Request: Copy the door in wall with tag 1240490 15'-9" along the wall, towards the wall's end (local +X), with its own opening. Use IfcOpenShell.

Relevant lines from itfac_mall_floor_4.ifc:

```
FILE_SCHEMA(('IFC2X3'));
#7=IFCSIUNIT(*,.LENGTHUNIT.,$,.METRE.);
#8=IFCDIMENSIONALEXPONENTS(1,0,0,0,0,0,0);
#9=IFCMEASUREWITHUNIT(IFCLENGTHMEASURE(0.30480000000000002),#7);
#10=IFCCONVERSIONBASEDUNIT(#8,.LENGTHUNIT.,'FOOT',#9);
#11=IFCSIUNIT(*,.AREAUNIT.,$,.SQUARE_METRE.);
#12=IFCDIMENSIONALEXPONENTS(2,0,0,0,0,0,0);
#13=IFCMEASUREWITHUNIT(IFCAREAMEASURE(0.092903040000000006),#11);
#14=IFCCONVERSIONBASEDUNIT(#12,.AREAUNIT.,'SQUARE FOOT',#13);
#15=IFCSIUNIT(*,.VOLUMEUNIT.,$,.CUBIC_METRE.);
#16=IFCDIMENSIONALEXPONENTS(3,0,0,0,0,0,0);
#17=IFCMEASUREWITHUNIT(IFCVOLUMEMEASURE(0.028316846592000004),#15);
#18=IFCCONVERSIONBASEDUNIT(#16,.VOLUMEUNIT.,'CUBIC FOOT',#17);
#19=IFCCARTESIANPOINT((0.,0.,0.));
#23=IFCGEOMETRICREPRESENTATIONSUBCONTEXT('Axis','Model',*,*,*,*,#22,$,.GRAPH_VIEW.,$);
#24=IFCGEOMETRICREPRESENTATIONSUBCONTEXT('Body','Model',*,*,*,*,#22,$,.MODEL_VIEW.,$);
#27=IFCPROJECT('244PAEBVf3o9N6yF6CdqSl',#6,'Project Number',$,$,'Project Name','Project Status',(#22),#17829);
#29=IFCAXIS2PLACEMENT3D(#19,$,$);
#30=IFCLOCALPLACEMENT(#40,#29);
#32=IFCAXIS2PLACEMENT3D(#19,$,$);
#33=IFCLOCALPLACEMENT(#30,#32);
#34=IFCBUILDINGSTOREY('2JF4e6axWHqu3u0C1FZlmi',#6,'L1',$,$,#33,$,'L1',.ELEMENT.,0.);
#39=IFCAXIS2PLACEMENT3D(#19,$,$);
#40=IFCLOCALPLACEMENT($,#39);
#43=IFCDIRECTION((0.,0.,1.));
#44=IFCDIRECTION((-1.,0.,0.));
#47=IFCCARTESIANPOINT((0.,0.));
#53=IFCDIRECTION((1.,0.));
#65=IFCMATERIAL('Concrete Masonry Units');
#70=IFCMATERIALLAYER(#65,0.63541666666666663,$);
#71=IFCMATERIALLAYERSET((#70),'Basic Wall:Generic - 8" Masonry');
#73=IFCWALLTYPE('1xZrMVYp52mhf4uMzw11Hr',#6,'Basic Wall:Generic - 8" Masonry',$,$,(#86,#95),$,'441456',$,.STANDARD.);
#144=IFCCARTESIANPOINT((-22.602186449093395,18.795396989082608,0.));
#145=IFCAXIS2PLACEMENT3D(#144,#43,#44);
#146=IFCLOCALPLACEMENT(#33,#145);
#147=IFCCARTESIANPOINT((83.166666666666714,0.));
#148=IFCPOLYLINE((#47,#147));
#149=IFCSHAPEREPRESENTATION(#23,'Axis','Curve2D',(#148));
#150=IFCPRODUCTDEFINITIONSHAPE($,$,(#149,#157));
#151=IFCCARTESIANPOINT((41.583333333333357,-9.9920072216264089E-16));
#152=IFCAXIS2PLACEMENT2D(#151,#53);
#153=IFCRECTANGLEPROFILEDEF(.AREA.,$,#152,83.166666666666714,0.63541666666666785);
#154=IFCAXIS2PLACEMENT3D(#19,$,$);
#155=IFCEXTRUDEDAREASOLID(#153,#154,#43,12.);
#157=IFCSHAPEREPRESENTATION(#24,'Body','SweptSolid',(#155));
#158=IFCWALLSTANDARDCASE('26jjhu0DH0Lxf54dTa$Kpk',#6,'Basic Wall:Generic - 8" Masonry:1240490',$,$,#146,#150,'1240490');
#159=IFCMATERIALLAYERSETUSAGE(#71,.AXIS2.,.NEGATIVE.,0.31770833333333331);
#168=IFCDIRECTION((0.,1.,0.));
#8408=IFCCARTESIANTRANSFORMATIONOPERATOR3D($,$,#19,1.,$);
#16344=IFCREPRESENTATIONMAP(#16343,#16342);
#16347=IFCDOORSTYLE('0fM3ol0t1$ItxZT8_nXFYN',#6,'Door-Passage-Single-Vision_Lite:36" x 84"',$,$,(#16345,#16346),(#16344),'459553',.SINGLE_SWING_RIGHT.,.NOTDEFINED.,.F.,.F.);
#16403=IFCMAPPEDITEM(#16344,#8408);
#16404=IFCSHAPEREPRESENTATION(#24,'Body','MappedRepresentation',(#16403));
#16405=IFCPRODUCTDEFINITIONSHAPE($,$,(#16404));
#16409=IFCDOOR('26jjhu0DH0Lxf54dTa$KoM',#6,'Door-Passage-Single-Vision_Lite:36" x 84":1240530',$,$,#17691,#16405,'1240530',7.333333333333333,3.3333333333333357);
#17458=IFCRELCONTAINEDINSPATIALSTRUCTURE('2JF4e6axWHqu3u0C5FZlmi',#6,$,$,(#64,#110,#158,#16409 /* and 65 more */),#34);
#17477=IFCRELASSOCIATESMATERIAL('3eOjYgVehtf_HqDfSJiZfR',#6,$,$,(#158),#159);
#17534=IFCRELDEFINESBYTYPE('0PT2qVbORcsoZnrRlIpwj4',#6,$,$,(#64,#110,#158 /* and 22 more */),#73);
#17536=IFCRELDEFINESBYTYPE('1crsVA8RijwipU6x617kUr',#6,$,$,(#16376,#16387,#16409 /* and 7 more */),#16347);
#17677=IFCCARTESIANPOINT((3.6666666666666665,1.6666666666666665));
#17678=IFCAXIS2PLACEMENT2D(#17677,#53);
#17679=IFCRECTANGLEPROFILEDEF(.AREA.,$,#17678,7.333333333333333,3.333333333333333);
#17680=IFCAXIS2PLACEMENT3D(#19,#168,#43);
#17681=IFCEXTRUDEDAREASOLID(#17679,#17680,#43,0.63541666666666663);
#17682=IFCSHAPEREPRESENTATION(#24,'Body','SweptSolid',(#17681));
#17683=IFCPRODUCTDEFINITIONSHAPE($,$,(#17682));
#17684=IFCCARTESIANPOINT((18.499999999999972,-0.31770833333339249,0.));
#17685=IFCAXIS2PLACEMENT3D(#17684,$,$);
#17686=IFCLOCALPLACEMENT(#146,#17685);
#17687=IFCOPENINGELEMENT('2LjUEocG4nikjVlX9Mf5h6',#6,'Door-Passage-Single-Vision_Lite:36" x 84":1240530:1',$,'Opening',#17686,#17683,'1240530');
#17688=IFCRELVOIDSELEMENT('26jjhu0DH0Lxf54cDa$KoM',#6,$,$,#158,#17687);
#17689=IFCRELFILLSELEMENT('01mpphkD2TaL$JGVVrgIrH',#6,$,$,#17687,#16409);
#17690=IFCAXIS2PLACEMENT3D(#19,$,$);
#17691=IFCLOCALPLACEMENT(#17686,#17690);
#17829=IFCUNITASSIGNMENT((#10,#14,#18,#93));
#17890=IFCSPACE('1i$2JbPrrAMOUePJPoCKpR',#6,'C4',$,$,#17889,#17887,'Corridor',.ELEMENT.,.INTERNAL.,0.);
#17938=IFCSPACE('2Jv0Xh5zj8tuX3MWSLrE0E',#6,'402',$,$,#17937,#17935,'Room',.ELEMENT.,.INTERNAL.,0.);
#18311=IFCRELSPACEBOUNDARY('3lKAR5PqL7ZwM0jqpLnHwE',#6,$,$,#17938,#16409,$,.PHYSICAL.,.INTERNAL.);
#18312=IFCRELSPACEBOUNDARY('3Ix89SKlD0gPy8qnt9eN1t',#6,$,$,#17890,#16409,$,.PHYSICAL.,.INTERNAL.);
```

```python
import ifcopenshell
import ifcopenshell.api.feature
import ifcopenshell.api.geometry
import ifcopenshell.api.root
import ifcopenshell.geom
import ifcopenshell.util.element
import ifcopenshell.util.placement
import ifcopenshell.util.shape
import ifcopenshell.util.unit

model = ifcopenshell.open("itfac_mall_floor_4.ifc")
unit_scale = ifcopenshell.util.unit.calculate_unit_scale(model)
settings = ifcopenshell.geom.settings()


def volume(element):
    """Net volume in cubic metres, openings subtracted."""
    shape = ifcopenshell.geom.create_shape(settings, element)
    return ifcopenshell.util.shape.get_volume(shape.geometry)


def reuse_history(source, copy):
    """copy_class also copies each property set's owner history, people and application; keep the originals."""
    for rel in copy.IsDefinedBy:
        if rel.is_a("IfcRelDefinesByProperties") and (history := rel.RelatingPropertyDefinition.OwnerHistory):
            rel.RelatingPropertyDefinition.OwnerHistory = source.OwnerHistory
            ifcopenshell.util.element.remove_deep2(model, history)


door = model.by_guid("26jjhu0DH0Lxf54dTa$KoM")
opening = door.FillsVoids[0].RelatingOpeningElement
wall = opening.VoidsElements[0].RelatingBuildingElement
before = volume(wall)
shift = ifcopenshell.util.placement.get_local_placement(wall.ObjectPlacement)[:3, 0] * 189 * 0.0254 / unit_scale

# copy_class copies the void relationship, type, container and properties, but no geometry.
new_opening = ifcopenshell.api.root.copy_class(model, product=opening)
new_opening.Representation = ifcopenshell.util.element.copy_deep(
    model, opening.Representation, exclude=["IfcGeometricRepresentationContext", "IfcRepresentationMap"]
)
new_opening.Name = 'Door-Passage-Single-Vision_Lite:36" x 84"'
new_opening.Tag = None
new_door = ifcopenshell.api.root.copy_class(model, product=door)
new_door.Representation = ifcopenshell.util.element.copy_deep(
    model, door.Representation, exclude=["IfcGeometricRepresentationContext", "IfcRepresentationMap"]
)
new_door.Name = 'Door-Passage-Single-Vision_Lite:36" x 84"'
new_door.Tag = None
reuse_history(door, new_door)
fills = ifcopenshell.api.feature.add_filling(model, opening=new_opening, element=new_door)
fills.OwnerHistory = new_door.OwnerHistory  # required in IFC2X3

for old, new in ((opening, new_opening), (door, new_door)):
    matrix = ifcopenshell.util.placement.get_local_placement(old.ObjectPlacement)
    matrix[:3, 3] += shift
    ifcopenshell.api.geometry.edit_object_placement(model, product=new, matrix=matrix, is_si=False)

after = volume(wall)

print(f"wall volume {before:.3f} -> {after:.3f} m3")

model.write("itfac_mall_floor_4_updated.ifc")
```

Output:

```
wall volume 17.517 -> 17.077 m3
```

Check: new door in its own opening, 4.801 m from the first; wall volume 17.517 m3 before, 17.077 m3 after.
